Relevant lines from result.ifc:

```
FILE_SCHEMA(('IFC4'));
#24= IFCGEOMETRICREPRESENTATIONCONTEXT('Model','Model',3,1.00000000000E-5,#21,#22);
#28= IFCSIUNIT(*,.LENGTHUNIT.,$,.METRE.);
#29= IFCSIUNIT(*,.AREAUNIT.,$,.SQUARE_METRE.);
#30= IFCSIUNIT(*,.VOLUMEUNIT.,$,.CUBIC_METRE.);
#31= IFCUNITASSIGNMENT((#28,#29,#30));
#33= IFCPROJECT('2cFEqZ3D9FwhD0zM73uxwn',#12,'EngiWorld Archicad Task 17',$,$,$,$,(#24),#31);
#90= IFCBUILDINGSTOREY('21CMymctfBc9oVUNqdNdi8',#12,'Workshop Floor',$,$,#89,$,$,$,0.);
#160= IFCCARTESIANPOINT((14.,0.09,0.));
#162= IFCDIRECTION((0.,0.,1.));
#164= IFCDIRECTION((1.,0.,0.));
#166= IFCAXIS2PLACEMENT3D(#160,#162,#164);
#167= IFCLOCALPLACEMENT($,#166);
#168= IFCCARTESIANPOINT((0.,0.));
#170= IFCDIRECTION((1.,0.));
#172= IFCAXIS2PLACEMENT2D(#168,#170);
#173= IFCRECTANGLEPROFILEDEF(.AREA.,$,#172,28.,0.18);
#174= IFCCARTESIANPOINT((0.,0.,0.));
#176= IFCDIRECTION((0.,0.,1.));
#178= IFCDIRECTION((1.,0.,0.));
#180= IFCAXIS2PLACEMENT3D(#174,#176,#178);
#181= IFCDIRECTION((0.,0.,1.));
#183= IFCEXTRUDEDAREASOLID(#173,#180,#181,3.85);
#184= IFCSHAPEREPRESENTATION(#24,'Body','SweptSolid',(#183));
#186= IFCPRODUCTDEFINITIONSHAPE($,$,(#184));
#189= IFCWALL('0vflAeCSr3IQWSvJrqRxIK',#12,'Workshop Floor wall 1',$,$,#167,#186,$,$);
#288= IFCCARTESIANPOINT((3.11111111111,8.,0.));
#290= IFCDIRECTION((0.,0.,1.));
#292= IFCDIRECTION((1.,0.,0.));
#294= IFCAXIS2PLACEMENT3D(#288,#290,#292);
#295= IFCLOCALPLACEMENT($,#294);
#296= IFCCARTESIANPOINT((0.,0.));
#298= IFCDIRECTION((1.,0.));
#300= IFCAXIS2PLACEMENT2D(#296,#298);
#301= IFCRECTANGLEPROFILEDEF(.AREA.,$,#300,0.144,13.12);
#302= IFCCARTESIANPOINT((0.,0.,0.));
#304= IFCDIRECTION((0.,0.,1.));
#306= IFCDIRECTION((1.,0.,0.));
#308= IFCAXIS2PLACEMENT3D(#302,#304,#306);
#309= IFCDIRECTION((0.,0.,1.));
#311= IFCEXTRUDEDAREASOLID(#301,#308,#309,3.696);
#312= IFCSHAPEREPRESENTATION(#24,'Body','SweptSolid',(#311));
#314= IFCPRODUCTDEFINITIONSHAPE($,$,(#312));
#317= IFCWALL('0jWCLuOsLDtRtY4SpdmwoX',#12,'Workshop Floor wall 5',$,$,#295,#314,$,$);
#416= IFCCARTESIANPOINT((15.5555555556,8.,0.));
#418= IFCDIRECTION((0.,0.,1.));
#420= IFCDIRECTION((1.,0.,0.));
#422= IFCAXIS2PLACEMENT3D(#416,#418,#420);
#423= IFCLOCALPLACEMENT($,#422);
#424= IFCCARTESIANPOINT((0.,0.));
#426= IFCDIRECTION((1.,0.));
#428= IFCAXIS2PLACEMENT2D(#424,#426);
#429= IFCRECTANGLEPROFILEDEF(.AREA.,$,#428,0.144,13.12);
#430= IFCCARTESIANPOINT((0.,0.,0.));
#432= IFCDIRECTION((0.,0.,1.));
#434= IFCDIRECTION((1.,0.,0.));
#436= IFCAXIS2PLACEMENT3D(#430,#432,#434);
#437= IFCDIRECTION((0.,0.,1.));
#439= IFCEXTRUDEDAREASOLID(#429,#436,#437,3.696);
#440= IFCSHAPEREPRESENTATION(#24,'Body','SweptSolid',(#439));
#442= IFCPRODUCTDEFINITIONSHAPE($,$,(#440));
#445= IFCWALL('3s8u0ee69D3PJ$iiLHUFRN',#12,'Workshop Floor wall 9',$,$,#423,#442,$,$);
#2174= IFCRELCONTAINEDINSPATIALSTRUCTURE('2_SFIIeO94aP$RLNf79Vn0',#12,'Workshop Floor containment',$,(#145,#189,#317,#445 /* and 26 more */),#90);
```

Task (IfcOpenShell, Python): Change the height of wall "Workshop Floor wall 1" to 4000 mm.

```python
import ifcopenshell
import ifcopenshell.geom
import ifcopenshell.util.shape
import ifcopenshell.util.unit

model = ifcopenshell.open("result.ifc")
unit_scale = ifcopenshell.util.unit.calculate_unit_scale(model)
settings = ifcopenshell.geom.settings()


def volume(element):
    """Net volume in cubic metres, openings subtracted."""
    shape = ifcopenshell.geom.create_shape(settings, element)
    return ifcopenshell.util.shape.get_volume(shape.geometry)


wall = model.by_id(189)
before = volume(wall)

body = next(r for r in wall.Representation.Representations if r.RepresentationIdentifier == "Body")
solid = body.Items[0]
old_height = solid.Depth
solid.Depth = 4 / unit_scale
after = volume(wall)

print(f"height {old_height:g} -> {solid.Depth:g}, volume {before:.3f} -> {after:.3f} m3")

model.write("result_v2.ifc")
```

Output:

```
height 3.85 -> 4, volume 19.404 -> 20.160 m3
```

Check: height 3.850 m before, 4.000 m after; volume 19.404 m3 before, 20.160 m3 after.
